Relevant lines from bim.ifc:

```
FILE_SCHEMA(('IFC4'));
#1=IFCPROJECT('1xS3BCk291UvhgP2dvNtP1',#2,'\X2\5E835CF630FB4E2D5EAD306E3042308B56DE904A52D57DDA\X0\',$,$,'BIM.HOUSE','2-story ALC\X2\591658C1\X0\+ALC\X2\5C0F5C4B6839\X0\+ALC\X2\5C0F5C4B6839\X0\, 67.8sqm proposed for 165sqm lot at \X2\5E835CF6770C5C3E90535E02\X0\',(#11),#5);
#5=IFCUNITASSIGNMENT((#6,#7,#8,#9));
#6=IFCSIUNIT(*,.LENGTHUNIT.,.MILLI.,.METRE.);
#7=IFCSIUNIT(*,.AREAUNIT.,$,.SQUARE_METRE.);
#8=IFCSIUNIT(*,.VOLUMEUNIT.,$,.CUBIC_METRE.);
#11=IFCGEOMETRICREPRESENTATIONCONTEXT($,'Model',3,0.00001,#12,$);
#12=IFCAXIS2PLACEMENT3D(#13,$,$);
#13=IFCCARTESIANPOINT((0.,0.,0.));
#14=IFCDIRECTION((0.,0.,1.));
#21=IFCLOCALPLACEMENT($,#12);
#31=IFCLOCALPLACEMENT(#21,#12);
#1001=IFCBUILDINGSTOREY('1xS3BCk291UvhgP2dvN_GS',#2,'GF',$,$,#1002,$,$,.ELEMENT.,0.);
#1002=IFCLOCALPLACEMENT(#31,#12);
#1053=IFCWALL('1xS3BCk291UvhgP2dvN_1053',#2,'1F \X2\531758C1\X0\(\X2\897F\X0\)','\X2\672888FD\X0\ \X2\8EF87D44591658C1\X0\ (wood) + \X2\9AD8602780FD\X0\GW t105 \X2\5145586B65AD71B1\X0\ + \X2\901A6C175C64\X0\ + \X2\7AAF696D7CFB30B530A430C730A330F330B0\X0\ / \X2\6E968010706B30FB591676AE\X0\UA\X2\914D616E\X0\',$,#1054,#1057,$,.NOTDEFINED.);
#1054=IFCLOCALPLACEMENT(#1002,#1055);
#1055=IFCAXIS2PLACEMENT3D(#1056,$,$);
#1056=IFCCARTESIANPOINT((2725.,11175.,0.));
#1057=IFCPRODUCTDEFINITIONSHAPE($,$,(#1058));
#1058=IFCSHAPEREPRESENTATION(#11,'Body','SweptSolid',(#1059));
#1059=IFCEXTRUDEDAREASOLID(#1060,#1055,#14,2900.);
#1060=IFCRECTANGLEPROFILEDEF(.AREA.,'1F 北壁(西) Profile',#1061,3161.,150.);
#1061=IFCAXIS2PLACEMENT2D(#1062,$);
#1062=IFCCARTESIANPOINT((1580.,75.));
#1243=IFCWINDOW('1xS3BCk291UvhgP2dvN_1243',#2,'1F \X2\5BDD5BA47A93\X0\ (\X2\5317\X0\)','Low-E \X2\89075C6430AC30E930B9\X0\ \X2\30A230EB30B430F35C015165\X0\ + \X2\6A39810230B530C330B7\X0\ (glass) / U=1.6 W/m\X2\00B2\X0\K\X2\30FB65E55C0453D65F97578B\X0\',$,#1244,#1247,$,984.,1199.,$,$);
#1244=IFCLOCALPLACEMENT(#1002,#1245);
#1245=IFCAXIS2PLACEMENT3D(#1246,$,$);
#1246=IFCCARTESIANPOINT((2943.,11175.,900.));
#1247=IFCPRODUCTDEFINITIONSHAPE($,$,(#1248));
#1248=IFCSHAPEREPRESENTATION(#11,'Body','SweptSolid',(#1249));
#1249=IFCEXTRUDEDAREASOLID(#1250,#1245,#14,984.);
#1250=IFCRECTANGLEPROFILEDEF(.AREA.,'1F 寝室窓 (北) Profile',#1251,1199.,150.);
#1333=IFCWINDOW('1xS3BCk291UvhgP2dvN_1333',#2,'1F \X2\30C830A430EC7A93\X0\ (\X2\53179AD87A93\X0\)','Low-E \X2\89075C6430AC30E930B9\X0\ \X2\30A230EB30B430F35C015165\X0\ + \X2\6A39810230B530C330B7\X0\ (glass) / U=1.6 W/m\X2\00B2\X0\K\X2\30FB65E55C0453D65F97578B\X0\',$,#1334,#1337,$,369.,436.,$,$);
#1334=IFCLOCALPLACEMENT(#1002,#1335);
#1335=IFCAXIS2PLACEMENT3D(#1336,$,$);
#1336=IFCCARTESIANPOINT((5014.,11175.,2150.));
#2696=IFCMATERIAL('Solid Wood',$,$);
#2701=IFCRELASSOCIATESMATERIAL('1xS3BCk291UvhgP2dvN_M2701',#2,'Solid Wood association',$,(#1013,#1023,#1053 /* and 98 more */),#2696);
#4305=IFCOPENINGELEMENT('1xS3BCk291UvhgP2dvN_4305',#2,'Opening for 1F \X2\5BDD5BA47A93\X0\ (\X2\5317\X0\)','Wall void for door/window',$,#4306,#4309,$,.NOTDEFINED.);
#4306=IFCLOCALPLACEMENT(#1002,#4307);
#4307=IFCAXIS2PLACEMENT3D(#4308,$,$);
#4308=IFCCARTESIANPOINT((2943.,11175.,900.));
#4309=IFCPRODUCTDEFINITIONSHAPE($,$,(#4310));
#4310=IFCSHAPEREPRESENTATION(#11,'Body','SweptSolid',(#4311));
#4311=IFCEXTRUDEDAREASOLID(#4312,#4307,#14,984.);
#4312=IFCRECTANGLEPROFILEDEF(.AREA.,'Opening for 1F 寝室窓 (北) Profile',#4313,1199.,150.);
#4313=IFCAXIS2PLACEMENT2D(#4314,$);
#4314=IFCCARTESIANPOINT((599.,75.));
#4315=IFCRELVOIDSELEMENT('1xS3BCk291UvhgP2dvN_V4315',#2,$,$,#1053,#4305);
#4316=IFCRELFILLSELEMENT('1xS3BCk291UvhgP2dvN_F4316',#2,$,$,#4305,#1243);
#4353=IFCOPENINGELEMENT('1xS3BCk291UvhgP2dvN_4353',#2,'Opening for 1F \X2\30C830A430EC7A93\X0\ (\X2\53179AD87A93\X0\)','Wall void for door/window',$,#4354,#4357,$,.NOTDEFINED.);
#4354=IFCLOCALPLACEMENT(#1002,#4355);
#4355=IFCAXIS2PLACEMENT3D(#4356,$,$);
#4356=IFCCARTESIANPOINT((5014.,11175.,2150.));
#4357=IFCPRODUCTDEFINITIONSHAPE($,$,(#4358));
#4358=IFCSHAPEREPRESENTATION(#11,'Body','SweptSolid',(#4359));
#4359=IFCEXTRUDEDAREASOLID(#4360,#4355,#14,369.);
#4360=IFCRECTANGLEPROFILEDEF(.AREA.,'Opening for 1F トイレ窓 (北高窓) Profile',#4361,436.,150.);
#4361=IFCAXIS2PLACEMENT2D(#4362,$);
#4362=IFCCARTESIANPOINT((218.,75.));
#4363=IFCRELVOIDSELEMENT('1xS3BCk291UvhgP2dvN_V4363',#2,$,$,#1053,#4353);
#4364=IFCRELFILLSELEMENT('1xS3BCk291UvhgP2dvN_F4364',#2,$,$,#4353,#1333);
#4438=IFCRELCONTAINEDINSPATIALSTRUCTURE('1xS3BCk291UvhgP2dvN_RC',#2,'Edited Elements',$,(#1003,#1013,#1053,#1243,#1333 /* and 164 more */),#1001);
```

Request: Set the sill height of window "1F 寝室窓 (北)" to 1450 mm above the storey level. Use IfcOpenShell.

```python
import numpy as np
import ifcopenshell
import ifcopenshell.api.geometry
import ifcopenshell.geom
import ifcopenshell.util.element
import ifcopenshell.util.placement
import ifcopenshell.util.shape
import ifcopenshell.util.unit

model = ifcopenshell.open("bim.ifc")
unit_scale = ifcopenshell.util.unit.calculate_unit_scale(model)

window = model.by_guid("1xS3BCk291UvhgP2dvN_1243")
opening = window.FillsVoids[0].RelatingOpeningElement
storey = ifcopenshell.util.element.get_container(window, ifc_class="IfcBuildingStorey")
level = ifcopenshell.util.placement.get_local_placement(storey.ObjectPlacement)[2, 3]

# The opening's origin need not be at the sill, so measure its lowest point.
shape = ifcopenshell.geom.create_shape(ifcopenshell.geom.settings(), opening)
bottom = ifcopenshell.util.shape.get_shape_bottom_elevation(shape, shape.geometry) / unit_scale
dz = level + 1450.0 - bottom

shift = np.array([0.0, 0.0, dz])
# The window is not placed relative to its opening, so move both.
for product in (opening, window):
    matrix = ifcopenshell.util.placement.get_local_placement(product.ObjectPlacement)
    matrix[:3, 3] += shift
    ifcopenshell.api.geometry.edit_object_placement(model, product=product, matrix=matrix, is_si=False)

print(f"moved by {dz * unit_scale:+.3f} m")

model.write("bim-out.ifc")
```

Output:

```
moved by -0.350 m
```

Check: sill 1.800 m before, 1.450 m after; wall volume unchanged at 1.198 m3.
